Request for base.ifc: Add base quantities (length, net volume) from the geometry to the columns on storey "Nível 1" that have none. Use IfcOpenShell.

First a look at what the model holds.

```python
import ifcopenshell
import ifcopenshell.util.element
import ifcopenshell.util.unit

model = ifcopenshell.open("base.ifc")
print(model.schema)
for unit_type in ("LENGTHUNIT", "AREAUNIT", "VOLUMEUNIT"):
    print(unit_type, ifcopenshell.util.unit.calculate_unit_scale(model, unit_type))
storey = next(s for s in model.by_type("IfcBuildingStorey") if s.Name == "Nível 1")
columns = [e for e in ifcopenshell.util.element.get_decomposition(storey) if e.is_a("IfcColumn")]
for e in sorted(columns, key=lambda e: e.id()):
    print(e.id(), e.is_a(), e.Name, list(ifcopenshell.util.element.get_psets(e, qtos_only=True)), sep=" | ")
```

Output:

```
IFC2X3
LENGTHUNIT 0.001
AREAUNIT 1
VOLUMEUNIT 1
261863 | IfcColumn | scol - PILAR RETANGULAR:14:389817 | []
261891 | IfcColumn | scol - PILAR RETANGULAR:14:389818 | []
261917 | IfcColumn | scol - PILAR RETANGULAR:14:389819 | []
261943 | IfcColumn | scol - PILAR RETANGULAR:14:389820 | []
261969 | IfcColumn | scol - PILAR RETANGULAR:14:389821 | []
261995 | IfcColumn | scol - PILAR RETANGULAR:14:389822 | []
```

```python
import ifcopenshell
import ifcopenshell.api.pset
import ifcopenshell.geom
import ifcopenshell.util.element
import ifcopenshell.util.shape
import ifcopenshell.util.unit

model = ifcopenshell.open("base.ifc")
unit_scale = ifcopenshell.util.unit.calculate_unit_scale(model)
volume_scale = ifcopenshell.util.unit.calculate_unit_scale(model, "VOLUMEUNIT")
settings = ifcopenshell.geom.settings()

storey = next(s for s in model.by_type("IfcBuildingStorey") if s.Name == "Nível 1")
columns = [e for e in ifcopenshell.util.element.get_decomposition(storey) if e.is_a("IfcColumn")]

for e in sorted(columns, key=lambda e: e.id()):
    if ifcopenshell.util.element.get_psets(e, qtos_only=True, should_inherit=False):
        continue
    # Geometry comes back in metres, in the element's own axes.
    shape = ifcopenshell.geom.create_shape(settings, e)
    values = {
        "Length": ifcopenshell.util.shape.get_z(shape.geometry) / unit_scale,
        "NetVolume": ifcopenshell.util.shape.get_volume(shape.geometry) / volume_scale,
    }
    qto = ifcopenshell.api.pset.add_qto(model, product=e, name="BaseQuantities")
    ifcopenshell.api.pset.edit_qto(model, qto=qto, properties=values)
    print(e.id(), {k: round(v, 3) for k, v in values.items()})

model.write("base-out.ifc")
```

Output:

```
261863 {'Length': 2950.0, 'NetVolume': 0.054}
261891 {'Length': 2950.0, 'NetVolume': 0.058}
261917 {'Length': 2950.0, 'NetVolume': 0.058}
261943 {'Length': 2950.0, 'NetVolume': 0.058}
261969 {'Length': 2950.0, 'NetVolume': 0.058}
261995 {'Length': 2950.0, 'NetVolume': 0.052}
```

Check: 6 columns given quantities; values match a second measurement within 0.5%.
